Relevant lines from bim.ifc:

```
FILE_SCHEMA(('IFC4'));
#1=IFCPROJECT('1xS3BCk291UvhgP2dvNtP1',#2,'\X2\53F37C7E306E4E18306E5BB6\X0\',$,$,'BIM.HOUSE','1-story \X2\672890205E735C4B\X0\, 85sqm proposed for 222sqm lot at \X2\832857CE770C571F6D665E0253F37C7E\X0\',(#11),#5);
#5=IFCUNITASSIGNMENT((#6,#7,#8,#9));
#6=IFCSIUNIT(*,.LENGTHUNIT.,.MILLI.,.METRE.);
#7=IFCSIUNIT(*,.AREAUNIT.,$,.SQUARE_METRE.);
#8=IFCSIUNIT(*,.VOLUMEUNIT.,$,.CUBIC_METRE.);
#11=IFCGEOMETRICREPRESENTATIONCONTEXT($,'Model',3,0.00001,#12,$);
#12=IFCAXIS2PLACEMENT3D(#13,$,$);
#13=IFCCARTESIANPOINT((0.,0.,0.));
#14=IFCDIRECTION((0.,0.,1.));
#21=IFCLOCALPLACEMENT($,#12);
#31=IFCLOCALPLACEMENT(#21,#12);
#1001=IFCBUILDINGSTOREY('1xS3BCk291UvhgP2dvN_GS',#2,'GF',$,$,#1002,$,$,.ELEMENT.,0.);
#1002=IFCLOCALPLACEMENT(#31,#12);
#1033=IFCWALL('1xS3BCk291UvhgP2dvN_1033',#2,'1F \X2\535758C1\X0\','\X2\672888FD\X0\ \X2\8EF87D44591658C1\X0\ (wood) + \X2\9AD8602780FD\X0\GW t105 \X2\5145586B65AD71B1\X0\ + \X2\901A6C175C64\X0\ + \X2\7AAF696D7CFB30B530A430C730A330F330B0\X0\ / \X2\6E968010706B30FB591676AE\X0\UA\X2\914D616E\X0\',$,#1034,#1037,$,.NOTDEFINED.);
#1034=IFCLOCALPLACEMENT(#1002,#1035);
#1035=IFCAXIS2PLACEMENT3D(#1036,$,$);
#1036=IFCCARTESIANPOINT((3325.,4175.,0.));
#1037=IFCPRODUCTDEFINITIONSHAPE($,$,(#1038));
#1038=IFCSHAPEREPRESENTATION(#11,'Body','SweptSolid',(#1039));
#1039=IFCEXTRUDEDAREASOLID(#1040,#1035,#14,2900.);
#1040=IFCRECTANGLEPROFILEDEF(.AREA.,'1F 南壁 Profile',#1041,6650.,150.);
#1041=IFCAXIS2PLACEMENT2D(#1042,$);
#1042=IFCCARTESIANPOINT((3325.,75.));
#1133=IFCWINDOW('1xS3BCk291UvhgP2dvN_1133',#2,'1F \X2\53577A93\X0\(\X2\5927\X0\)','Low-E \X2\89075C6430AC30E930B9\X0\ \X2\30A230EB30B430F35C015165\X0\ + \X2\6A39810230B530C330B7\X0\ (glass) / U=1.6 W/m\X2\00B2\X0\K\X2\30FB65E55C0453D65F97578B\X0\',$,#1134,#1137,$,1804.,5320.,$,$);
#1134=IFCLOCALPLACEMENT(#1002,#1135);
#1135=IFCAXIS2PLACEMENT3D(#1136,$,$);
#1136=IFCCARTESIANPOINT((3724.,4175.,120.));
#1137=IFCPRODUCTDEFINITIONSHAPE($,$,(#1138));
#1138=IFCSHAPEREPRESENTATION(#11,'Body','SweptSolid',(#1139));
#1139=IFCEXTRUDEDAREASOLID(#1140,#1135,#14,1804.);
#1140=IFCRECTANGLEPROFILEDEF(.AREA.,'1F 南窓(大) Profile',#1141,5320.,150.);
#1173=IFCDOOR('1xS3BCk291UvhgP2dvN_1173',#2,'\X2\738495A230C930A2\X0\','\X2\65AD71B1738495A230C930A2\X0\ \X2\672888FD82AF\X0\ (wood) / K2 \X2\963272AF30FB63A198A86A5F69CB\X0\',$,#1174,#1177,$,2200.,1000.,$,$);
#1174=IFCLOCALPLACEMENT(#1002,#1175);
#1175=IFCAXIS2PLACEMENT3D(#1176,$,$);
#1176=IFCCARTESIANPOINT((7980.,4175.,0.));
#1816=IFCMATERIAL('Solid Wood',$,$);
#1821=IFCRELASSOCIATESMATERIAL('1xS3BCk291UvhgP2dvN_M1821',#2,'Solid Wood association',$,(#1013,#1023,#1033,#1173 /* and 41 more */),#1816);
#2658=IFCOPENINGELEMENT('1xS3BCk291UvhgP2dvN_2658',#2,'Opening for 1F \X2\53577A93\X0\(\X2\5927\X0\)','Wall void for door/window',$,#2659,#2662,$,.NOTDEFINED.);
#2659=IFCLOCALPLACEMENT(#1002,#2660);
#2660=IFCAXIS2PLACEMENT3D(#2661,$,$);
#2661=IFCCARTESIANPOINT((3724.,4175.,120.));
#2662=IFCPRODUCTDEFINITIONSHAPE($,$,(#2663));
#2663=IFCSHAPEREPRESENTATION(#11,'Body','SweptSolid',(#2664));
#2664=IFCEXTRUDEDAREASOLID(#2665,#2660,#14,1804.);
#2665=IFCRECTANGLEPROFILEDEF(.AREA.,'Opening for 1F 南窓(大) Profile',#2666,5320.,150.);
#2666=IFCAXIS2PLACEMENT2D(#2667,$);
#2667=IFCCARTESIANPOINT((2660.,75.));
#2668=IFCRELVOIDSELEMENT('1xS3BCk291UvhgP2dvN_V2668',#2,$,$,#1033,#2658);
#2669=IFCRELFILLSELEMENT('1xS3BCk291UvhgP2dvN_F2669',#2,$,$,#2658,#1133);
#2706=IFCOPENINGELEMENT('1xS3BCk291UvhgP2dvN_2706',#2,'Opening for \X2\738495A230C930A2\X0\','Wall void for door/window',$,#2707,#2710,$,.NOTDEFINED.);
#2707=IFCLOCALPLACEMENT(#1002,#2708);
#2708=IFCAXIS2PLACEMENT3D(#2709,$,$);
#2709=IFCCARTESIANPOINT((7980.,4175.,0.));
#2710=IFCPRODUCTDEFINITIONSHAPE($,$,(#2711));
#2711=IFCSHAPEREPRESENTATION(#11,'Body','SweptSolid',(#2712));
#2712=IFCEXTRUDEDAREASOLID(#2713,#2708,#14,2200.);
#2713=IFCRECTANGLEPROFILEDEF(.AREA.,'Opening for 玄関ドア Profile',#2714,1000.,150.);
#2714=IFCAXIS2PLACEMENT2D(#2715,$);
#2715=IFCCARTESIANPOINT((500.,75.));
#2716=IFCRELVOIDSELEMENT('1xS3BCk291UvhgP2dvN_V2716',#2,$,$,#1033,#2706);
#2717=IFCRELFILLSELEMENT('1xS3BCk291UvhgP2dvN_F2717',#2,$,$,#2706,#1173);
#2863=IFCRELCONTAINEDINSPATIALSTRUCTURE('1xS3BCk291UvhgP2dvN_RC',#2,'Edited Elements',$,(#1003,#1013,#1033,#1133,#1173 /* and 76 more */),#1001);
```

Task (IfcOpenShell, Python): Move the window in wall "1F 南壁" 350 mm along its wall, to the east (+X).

```python
import ifcopenshell
import ifcopenshell.api.geometry
import ifcopenshell.util.placement

model = ifcopenshell.open("bim.ifc")

window = model.by_id(1133)
opening = window.FillsVoids[0].RelatingOpeningElement
wall = opening.VoidsElements[0].RelatingBuildingElement

wall_matrix = ifcopenshell.util.placement.get_local_placement(wall.ObjectPlacement)
shift = wall_matrix[:3, 0] * 350.0
before = ifcopenshell.util.placement.get_local_placement(window.ObjectPlacement)[:3, 3].copy()

# The window is not placed relative to its opening, so move both.
for product in (opening, window):
    matrix = ifcopenshell.util.placement.get_local_placement(product.ObjectPlacement)
    matrix[:3, 3] += shift
    ifcopenshell.api.geometry.edit_object_placement(model, product=product, matrix=matrix, is_si=False)

after = ifcopenshell.util.placement.get_local_placement(window.ObjectPlacement)[:3, 3]
print("window moved by", (after - before).round(3) + 0.0)

model.write("bim_updated.ifc")
```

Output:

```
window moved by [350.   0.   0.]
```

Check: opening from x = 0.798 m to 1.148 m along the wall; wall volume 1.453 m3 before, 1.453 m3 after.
